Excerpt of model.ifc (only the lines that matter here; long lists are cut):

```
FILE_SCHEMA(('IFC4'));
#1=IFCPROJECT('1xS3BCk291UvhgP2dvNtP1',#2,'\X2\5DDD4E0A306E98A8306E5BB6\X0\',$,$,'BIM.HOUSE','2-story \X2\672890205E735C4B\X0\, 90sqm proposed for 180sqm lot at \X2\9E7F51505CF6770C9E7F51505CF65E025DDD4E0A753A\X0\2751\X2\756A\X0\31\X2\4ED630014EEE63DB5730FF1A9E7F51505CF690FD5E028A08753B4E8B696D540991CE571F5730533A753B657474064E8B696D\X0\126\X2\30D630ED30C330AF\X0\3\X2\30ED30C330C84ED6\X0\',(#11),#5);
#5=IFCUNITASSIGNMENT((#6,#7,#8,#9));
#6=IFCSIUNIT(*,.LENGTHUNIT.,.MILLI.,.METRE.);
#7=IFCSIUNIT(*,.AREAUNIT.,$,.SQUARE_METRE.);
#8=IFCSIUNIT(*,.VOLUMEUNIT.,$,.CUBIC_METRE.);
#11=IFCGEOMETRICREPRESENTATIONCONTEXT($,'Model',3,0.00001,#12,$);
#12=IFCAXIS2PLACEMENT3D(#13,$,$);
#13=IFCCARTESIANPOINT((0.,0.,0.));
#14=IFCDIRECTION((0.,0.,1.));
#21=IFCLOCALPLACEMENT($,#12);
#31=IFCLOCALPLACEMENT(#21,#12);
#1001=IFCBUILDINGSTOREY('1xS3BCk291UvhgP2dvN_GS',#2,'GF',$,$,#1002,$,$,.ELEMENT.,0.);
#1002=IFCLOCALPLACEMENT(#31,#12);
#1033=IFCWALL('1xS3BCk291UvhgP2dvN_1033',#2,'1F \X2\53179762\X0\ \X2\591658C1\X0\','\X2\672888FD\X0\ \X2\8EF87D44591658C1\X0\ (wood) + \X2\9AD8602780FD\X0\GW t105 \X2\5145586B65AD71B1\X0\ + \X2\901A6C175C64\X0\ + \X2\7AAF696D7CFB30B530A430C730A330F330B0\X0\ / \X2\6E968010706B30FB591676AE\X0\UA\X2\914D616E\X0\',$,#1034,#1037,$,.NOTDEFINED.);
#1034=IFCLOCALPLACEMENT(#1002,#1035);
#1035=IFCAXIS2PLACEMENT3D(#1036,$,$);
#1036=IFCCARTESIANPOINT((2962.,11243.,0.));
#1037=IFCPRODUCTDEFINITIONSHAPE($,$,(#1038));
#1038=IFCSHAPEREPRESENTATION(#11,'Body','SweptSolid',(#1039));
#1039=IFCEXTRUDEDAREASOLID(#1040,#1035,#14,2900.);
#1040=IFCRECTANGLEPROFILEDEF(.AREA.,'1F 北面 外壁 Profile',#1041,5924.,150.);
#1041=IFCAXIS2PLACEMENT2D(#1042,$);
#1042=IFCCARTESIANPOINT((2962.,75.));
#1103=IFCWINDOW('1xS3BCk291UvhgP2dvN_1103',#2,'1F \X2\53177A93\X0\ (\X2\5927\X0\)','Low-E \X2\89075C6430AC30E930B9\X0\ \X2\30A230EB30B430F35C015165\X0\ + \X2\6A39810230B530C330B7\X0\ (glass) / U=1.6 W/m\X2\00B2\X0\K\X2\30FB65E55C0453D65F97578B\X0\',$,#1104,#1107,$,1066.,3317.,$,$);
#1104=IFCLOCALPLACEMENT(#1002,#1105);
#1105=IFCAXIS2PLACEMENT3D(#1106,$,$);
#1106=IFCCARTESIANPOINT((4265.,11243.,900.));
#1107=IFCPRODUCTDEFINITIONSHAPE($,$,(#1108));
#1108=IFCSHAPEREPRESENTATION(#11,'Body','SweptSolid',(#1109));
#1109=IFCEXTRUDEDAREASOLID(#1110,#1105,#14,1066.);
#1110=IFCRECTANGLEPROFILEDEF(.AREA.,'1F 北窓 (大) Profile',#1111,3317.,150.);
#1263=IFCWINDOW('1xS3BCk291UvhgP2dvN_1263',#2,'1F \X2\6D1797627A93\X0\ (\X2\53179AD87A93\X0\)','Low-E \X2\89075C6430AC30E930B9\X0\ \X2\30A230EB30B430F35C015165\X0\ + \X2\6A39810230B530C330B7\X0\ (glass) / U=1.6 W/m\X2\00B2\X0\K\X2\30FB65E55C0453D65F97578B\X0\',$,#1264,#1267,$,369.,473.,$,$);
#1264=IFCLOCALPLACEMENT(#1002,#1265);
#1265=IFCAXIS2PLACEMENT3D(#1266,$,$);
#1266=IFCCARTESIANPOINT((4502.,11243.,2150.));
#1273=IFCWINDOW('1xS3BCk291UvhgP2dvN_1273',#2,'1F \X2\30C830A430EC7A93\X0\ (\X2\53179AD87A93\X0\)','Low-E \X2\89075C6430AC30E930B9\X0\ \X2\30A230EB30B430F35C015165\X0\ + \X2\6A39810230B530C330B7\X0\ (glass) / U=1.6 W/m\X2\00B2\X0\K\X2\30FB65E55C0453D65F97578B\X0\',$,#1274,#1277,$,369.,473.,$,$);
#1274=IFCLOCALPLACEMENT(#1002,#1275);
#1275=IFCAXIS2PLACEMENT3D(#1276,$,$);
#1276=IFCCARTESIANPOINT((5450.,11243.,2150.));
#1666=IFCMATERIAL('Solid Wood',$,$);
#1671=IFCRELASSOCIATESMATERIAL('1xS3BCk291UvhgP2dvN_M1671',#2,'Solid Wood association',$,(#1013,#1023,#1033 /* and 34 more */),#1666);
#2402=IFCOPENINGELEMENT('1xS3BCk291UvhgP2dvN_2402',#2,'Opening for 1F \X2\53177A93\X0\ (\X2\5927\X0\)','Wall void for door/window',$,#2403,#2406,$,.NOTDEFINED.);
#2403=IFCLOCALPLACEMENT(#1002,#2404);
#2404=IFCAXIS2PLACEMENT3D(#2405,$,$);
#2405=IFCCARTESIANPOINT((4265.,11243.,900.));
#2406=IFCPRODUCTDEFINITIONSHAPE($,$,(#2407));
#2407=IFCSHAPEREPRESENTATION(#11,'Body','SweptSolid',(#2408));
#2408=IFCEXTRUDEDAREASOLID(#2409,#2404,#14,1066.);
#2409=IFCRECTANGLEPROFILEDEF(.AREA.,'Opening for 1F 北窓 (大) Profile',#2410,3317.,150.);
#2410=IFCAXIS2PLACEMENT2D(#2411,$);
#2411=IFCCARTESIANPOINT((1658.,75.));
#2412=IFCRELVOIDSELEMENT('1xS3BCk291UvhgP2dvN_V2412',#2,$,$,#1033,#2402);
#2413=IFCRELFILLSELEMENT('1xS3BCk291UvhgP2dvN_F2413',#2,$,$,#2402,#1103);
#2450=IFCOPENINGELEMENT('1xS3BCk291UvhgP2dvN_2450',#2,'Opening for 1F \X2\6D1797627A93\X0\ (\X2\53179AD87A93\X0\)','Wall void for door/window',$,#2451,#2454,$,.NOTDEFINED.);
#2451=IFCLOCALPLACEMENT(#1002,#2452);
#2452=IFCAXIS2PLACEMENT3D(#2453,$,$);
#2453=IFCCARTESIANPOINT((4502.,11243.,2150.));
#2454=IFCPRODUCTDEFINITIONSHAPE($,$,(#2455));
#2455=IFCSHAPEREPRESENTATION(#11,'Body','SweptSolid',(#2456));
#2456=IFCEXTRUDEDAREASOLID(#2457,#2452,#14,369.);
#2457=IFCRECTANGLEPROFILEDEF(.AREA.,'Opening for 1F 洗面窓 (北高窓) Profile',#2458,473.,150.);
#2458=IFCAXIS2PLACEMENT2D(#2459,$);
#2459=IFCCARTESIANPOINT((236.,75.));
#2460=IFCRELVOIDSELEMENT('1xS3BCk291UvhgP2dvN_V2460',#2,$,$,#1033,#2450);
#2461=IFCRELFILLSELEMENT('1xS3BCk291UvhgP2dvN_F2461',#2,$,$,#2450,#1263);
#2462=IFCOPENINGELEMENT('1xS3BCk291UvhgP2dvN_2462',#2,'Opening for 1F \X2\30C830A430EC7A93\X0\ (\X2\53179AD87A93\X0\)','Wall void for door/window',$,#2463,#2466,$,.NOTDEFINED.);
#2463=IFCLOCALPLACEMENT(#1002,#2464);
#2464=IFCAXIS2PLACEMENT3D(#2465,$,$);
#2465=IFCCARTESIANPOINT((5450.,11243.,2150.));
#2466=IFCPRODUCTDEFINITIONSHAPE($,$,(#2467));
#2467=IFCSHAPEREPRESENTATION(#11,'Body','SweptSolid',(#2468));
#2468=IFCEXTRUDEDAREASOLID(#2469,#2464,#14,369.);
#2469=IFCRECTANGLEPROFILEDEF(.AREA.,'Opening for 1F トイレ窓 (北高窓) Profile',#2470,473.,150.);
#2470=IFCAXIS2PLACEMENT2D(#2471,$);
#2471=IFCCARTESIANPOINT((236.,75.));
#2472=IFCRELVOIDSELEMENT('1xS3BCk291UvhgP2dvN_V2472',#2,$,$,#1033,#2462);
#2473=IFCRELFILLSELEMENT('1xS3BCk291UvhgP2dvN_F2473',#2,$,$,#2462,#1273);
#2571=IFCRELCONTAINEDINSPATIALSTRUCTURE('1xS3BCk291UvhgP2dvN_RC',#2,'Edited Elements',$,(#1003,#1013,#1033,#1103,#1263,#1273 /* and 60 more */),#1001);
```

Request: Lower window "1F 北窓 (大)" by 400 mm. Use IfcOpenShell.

```python
import numpy as np
import ifcopenshell
import ifcopenshell.api.geometry
import ifcopenshell.util.placement
import ifcopenshell.util.unit

model = ifcopenshell.open("model.ifc")
unit_scale = ifcopenshell.util.unit.calculate_unit_scale(model)

window = model.by_guid("1xS3BCk291UvhgP2dvN_1103")
opening = window.FillsVoids[0].RelatingOpeningElement
dz = -400.0

shift = np.array([0.0, 0.0, dz])
# The window is not placed relative to its opening, so move both.
for product in (opening, window):
    matrix = ifcopenshell.util.placement.get_local_placement(product.ObjectPlacement)
    matrix[:3, 3] += shift
    ifcopenshell.api.geometry.edit_object_placement(model, product=product, matrix=matrix, is_si=False)

print(f"moved by {dz * unit_scale:+.3f} m")

model.write("model_updated.ifc")
```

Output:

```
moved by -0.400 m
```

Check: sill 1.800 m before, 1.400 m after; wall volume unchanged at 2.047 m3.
